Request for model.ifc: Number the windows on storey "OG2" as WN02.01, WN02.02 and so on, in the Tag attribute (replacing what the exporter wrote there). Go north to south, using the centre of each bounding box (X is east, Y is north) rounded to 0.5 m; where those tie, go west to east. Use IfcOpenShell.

First a look at what the model holds.

```python
import ifcopenshell
import ifcopenshell.util.element
import ifcopenshell.util.placement

model = ifcopenshell.open("model.ifc")
print(model.schema)
storey = next(s for s in model.by_type("IfcBuildingStorey") if s.Name == "OG2")
windows = [e for e in ifcopenshell.util.element.get_decomposition(storey) if e.is_a("IfcWindow")]
for e in sorted(windows, key=lambda e: e.id()):
    origin = ifcopenshell.util.placement.get_local_placement(e.ObjectPlacement)[:3, 3]
    print(e.id(), e.Tag, e.Name, origin.round(2) + 0.0, sep=" | ")
```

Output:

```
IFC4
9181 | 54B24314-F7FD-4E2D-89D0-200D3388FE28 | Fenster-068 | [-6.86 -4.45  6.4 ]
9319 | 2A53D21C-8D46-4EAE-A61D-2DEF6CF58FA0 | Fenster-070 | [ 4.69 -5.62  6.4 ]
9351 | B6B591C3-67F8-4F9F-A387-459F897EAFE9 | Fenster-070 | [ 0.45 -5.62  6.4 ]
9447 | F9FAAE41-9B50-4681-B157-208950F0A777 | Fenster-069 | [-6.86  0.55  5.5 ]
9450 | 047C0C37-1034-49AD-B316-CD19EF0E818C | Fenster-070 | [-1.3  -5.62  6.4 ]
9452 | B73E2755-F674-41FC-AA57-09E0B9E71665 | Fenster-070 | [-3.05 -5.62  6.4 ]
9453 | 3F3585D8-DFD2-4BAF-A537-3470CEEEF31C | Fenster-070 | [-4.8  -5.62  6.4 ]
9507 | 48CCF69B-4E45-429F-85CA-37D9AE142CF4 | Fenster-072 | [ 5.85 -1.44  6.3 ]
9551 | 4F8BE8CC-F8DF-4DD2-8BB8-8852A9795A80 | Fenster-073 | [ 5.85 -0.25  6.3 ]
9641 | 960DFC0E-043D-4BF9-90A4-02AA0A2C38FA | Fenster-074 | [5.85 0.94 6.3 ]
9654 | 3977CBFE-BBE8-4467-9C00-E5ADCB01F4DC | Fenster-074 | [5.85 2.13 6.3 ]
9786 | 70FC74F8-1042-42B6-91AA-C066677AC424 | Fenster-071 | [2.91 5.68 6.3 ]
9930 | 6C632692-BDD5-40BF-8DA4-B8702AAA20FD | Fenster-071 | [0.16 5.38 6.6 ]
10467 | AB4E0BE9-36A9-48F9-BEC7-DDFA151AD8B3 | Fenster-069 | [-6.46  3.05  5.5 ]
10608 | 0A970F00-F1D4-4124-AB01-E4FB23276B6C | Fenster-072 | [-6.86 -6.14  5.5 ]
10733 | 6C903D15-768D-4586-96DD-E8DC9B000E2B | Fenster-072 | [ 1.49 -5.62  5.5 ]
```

```python
import ifcopenshell
import ifcopenshell.geom
import ifcopenshell.util.element
import ifcopenshell.util.shape

model = ifcopenshell.open("model.ifc")
settings = ifcopenshell.geom.settings()
settings.set("use-world-coords", True)


def centre(element):
    shape = ifcopenshell.geom.create_shape(settings, element)
    return ifcopenshell.util.shape.get_bbox_centroid(shape.geometry)


storey = next(s for s in model.by_type("IfcBuildingStorey") if s.Name == "OG2")
windows = [e for e in ifcopenshell.util.element.get_decomposition(storey) if e.is_a("IfcWindow")]

# Insertion points can sit at a corner or the storey origin, so sort by the geometry (in metres).
centres = {e: centre(e) for e in windows}
windows.sort(key=lambda e: (-round(centres[e][1] / 0.5), centres[e][0]))

for i, e in enumerate(windows, start=1):
    number = f"WN02.{i:02d}"
    e.Tag = number
    print(e.id(), number)

model.write("model-out.ifc")
```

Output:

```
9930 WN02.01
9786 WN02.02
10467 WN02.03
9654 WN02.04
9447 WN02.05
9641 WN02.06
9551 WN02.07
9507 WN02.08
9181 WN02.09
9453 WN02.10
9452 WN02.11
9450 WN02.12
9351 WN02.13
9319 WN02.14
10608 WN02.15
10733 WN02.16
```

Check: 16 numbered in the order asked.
